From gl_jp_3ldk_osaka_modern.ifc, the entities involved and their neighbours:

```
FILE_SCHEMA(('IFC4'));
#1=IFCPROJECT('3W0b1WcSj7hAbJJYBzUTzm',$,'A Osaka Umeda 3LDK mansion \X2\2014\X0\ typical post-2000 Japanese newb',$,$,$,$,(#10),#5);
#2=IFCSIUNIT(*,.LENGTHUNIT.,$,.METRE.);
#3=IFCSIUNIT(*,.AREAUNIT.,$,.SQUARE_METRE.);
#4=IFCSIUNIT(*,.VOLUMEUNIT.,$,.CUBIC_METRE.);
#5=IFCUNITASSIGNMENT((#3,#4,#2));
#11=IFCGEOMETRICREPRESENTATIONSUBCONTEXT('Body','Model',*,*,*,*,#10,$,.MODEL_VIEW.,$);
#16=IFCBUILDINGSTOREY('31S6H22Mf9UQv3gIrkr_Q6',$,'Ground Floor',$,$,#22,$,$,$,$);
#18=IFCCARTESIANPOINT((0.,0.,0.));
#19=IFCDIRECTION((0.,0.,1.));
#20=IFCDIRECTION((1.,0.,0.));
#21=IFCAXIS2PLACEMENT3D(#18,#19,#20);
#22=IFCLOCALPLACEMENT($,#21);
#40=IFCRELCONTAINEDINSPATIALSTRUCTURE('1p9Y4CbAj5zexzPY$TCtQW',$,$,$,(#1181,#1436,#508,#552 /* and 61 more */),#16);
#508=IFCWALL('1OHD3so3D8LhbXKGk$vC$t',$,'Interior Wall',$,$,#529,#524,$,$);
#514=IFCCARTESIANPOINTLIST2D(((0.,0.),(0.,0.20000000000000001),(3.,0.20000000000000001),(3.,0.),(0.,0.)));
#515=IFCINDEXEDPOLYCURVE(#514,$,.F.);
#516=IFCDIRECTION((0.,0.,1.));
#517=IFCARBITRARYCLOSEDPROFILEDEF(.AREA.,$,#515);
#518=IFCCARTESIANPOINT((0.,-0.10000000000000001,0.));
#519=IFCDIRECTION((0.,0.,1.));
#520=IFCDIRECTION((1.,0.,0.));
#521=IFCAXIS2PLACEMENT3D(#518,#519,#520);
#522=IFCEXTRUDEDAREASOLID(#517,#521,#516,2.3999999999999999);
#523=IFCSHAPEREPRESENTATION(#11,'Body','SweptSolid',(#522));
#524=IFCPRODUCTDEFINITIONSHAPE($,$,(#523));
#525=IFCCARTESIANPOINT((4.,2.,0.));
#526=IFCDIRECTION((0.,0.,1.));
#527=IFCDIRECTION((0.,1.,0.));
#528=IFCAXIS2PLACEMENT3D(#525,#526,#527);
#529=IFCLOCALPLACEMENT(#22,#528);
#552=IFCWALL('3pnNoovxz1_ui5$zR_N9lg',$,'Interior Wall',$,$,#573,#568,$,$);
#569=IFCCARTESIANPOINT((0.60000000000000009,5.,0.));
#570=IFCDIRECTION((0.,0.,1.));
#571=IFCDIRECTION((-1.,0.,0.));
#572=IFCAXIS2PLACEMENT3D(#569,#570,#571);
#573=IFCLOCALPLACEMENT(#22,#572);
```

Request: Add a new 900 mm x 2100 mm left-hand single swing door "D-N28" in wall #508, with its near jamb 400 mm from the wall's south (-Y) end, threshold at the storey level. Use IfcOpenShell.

```python
import numpy as np
import ifcopenshell
import ifcopenshell.api.feature
import ifcopenshell.api.geometry
import ifcopenshell.api.root
import ifcopenshell.api.spatial
import ifcopenshell.geom
import ifcopenshell.util.element
import ifcopenshell.util.placement
import ifcopenshell.util.representation
import ifcopenshell.util.shape
import ifcopenshell.util.unit

model = ifcopenshell.open("gl_jp_3ldk_osaka_modern.ifc")
unit_scale = ifcopenshell.util.unit.calculate_unit_scale(model)
settings = ifcopenshell.geom.settings()


def volume(element):
    """Net volume in cubic metres, openings subtracted."""
    shape = ifcopenshell.geom.create_shape(settings, element)
    return ifcopenshell.util.shape.get_volume(shape.geometry)


wall = model.by_id(508)
storey = ifcopenshell.util.element.get_container(wall, ifc_class="IfcBuildingStorey")
context = ifcopenshell.util.representation.get_context(model, "Model", "Body", "MODEL_VIEW")
before = volume(wall)

width, height, from_end, sill = 0.9, 2.1, 0.4, 0.0  # metres

# The wall runs along its own X axis, and the end named is its -X end.
wall_shape = ifcopenshell.geom.create_shape(settings, wall)
x, y, z = ifcopenshell.util.shape.get_vertices(wall_shape.geometry).T
start = x.min() + from_end
face, thickness = float(y.min()), float(y.max() - y.min())
wall_matrix = ifcopenshell.util.placement.get_local_placement(wall.ObjectPlacement)
level = ifcopenshell.util.placement.get_local_placement(storey.ObjectPlacement)[2, 3]


def in_wall(x, y):
    """Placement at x, y metres in the wall's axes, at sill height."""
    matrix = wall_matrix.copy()
    matrix[:, 3] = wall_matrix @ np.array([x / unit_scale, y / unit_scale, 0.0, 1.0])
    matrix[2, 3] = level + sill / unit_scale
    return matrix


# Opening: a box that overshoots both wall faces by 50 mm.
opening = ifcopenshell.api.root.create_entity(model, ifc_class="IfcOpeningElement", predefined_type="OPENING")
box = ifcopenshell.api.geometry.add_wall_representation(
    model, context=context, length=width, height=height, thickness=thickness + 0.1
)
ifcopenshell.api.geometry.assign_representation(model, product=opening, representation=box)
ifcopenshell.api.geometry.edit_object_placement(model, product=opening, matrix=in_wall(start, face - 0.05), is_si=False)
ifcopenshell.api.feature.add_feature(model, feature=opening, element=wall)

door = ifcopenshell.api.root.create_entity(model, ifc_class="IfcDoor", name="D-N28", predefined_type="DOOR")
door.OverallWidth, door.OverallHeight = width / unit_scale, height / unit_scale
door.OperationType = "SINGLE_SWING_LEFT"
body = ifcopenshell.api.geometry.add_door_representation(
    model,
    context=context,
    overall_width=door.OverallWidth,
    overall_height=door.OverallHeight,
    operation_type="SINGLE_SWING_LEFT",
    lining_properties={"LiningDepth": thickness / unit_scale, "ThresholdDepth": thickness / unit_scale},
)
ifcopenshell.api.geometry.assign_representation(model, product=door, representation=body)
ifcopenshell.api.spatial.assign_container(model, products=[door], relating_structure=storey)
ifcopenshell.api.feature.add_filling(model, opening=opening, element=door)

# The lining spans the wall, so the door starts at the wall face.
ifcopenshell.api.geometry.edit_object_placement(model, product=door, matrix=in_wall(start, face), is_si=False)

after = volume(wall)

print(f"wall volume {before:.3f} -> {after:.3f} m3")

model.write("gl_jp_3ldk_osaka_modern-out.ifc")
```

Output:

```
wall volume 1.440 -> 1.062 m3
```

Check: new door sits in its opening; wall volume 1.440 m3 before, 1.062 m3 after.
